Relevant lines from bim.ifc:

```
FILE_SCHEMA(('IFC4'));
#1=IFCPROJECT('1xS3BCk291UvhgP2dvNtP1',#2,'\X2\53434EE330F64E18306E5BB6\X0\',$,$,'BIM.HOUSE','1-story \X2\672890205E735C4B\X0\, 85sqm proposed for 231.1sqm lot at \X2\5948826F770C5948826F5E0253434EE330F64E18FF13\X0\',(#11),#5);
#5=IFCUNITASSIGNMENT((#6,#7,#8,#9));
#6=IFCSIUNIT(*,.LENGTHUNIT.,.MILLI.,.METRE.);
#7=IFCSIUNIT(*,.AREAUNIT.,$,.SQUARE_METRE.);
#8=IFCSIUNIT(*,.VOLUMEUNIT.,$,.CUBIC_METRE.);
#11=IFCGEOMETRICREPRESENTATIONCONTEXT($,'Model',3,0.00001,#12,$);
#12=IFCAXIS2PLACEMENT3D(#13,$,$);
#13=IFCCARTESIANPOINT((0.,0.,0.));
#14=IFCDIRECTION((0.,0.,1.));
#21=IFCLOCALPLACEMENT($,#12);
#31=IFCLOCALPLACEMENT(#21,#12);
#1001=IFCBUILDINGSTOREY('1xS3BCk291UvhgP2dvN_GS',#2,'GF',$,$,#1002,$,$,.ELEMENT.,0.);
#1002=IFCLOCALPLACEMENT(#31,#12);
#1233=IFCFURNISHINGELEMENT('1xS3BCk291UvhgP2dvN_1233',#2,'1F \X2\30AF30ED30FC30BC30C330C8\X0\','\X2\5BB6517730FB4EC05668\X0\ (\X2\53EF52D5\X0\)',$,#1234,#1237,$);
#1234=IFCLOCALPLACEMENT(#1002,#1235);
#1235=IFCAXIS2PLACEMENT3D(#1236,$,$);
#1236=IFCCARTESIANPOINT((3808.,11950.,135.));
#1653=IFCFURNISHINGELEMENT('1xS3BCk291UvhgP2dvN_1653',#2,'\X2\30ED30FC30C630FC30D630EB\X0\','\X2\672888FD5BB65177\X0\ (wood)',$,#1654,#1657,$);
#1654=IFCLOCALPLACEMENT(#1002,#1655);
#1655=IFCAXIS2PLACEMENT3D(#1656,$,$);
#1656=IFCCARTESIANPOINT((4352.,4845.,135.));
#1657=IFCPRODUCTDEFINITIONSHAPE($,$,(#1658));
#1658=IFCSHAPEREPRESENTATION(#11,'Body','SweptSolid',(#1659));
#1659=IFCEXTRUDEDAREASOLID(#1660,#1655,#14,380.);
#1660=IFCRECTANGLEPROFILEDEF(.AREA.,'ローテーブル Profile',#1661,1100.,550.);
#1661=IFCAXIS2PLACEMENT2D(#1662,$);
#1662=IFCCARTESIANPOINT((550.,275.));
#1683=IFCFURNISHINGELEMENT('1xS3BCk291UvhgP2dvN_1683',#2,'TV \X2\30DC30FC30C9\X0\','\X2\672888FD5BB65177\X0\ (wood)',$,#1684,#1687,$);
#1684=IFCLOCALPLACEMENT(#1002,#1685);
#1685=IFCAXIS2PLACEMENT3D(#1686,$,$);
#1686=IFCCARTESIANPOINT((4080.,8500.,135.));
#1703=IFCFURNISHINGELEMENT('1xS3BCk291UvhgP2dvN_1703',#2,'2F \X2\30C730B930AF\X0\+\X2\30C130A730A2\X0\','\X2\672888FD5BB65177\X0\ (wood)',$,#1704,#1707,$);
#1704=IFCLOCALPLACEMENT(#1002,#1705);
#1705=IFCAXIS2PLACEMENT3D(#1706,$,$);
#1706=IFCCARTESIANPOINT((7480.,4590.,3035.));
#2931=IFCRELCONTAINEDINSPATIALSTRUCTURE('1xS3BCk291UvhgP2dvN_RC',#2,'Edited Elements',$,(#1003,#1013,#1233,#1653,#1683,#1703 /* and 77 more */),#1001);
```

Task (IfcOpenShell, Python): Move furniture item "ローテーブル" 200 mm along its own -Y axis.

```python
import ifcopenshell
import ifcopenshell.api.geometry
import ifcopenshell.util.placement
import ifcopenshell.util.unit

model = ifcopenshell.open("bim.ifc")
unit_scale = ifcopenshell.util.unit.calculate_unit_scale(model)

item = model.by_guid("1xS3BCk291UvhgP2dvN_1653")
matrix = ifcopenshell.util.placement.get_local_placement(item.ObjectPlacement)
matrix[:3, 3] -= matrix[:3, 1] * 0.2 / unit_scale
ifcopenshell.api.geometry.edit_object_placement(model, product=item, matrix=matrix, is_si=False)

print(ifcopenshell.util.placement.get_local_placement(item.ObjectPlacement).round(3) + 0.0)

model.write("bim_edited.ifc")
```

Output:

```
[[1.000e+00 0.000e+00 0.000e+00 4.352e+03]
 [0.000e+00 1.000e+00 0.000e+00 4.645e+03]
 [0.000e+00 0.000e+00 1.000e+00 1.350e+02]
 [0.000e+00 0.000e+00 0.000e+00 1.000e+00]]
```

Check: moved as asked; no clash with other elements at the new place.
